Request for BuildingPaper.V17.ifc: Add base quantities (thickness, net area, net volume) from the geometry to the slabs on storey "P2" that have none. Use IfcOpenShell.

First a look at what the model holds.

```python
import ifcopenshell
import ifcopenshell.util.element
import ifcopenshell.util.unit

model = ifcopenshell.open("BuildingPaper.V17.ifc")
print(model.schema)
for unit_type in ("LENGTHUNIT", "AREAUNIT", "VOLUMEUNIT"):
    print(unit_type, ifcopenshell.util.unit.calculate_unit_scale(model, unit_type))
storey = next(s for s in model.by_type("IfcBuildingStorey") if s.Name == "P2")
slabs = [e for e in ifcopenshell.util.element.get_decomposition(storey) if e.is_a("IfcSlab")]
for e in sorted(slabs, key=lambda e: e.id()):
    print(e.id(), e.is_a(), e.Name, list(ifcopenshell.util.element.get_psets(e, qtos_only=True)), sep=" | ")
```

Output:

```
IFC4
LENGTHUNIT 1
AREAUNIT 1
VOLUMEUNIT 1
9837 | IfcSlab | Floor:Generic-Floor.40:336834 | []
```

```python
import ifcopenshell
import ifcopenshell.api.pset
import ifcopenshell.geom
import ifcopenshell.util.element
import ifcopenshell.util.shape
import ifcopenshell.util.unit

model = ifcopenshell.open("BuildingPaper.V17.ifc")
unit_scale = ifcopenshell.util.unit.calculate_unit_scale(model)
area_scale = ifcopenshell.util.unit.calculate_unit_scale(model, "AREAUNIT")
volume_scale = ifcopenshell.util.unit.calculate_unit_scale(model, "VOLUMEUNIT")
settings = ifcopenshell.geom.settings()

storey = next(s for s in model.by_type("IfcBuildingStorey") if s.Name == "P2")
slabs = [e for e in ifcopenshell.util.element.get_decomposition(storey) if e.is_a("IfcSlab")]

for e in sorted(slabs, key=lambda e: e.id()):
    if ifcopenshell.util.element.get_psets(e, qtos_only=True, should_inherit=False):
        continue
    # Geometry comes back in metres, in the element's own axes.
    shape = ifcopenshell.geom.create_shape(settings, e)
    values = {
        "Width": ifcopenshell.util.shape.get_z(shape.geometry) / unit_scale,
        "NetArea": ifcopenshell.util.shape.get_footprint_area(shape.geometry) / area_scale,
        "NetVolume": ifcopenshell.util.shape.get_volume(shape.geometry) / volume_scale,
    }
    qto = ifcopenshell.api.pset.add_qto(model, product=e, name="Qto_SlabBaseQuantities")
    ifcopenshell.api.pset.edit_qto(model, qto=qto, properties=values)
    print(e.id(), {k: round(v, 3) for k, v in values.items()})

model.write("BuildingPaper.V17_edited.ifc")
```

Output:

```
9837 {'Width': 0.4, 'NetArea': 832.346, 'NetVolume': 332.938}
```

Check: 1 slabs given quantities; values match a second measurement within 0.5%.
